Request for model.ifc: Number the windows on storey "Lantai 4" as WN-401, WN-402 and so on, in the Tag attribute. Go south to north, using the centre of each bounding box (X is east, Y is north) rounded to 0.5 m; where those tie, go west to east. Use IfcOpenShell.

First a look at what the model holds.

```python
import ifcopenshell
import ifcopenshell.util.element
import ifcopenshell.util.placement

model = ifcopenshell.open("model.ifc")
print(model.schema)
storey = next(s for s in model.by_type("IfcBuildingStorey") if s.Name == "Lantai 4")
windows = [e for e in ifcopenshell.util.element.get_decomposition(storey) if e.is_a("IfcWindow")]
for e in sorted(windows, key=lambda e: e.id()):
    origin = ifcopenshell.util.placement.get_local_placement(e.ObjectPlacement)[:3, 3]
    print(e.id(), e.Tag, e.Name, origin.round(2) + 0.0, sep=" | ")
```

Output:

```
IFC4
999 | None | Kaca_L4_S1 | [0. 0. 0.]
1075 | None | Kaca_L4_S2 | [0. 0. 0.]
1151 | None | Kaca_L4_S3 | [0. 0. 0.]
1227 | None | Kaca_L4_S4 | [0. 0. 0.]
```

```python
import ifcopenshell
import ifcopenshell.geom
import ifcopenshell.util.element
import ifcopenshell.util.shape

model = ifcopenshell.open("model.ifc")
settings = ifcopenshell.geom.settings()
settings.set("use-world-coords", True)


def centre(element):
    shape = ifcopenshell.geom.create_shape(settings, element)
    return ifcopenshell.util.shape.get_bbox_centroid(shape.geometry)


storey = next(s for s in model.by_type("IfcBuildingStorey") if s.Name == "Lantai 4")
windows = [e for e in ifcopenshell.util.element.get_decomposition(storey) if e.is_a("IfcWindow")]

# Insertion points can sit at a corner or the storey origin, so sort by the geometry (in metres).
centres = {e: centre(e) for e in windows}
windows.sort(key=lambda e: (round(centres[e][1] / 0.5), centres[e][0]))

for i, e in enumerate(windows, start=1):
    number = f"WN-4{i:02d}"
    e.Tag = number
    print(e.id(), number)

model.write("model_rev.ifc")
```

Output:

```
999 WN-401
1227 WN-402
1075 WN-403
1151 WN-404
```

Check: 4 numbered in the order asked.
